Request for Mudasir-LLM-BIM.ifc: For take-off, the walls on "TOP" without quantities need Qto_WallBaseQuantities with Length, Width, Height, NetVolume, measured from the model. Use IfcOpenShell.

First a look at what the model holds.

```python
import ifcopenshell
import ifcopenshell.util.element
import ifcopenshell.util.unit

model = ifcopenshell.open("Mudasir-LLM-BIM.ifc")
print(model.schema)
for unit_type in ("LENGTHUNIT", "AREAUNIT", "VOLUMEUNIT"):
    print(unit_type, ifcopenshell.util.unit.calculate_unit_scale(model, unit_type))
storey = next(s for s in model.by_type("IfcBuildingStorey") if s.Name == "TOP")
walls = [e for e in ifcopenshell.util.element.get_decomposition(storey) if e.is_a("IfcWall")]
for e in sorted(walls, key=lambda e: e.id()):
    print(e.id(), e.is_a(), e.Name, list(ifcopenshell.util.element.get_psets(e, qtos_only=True)), sep=" | ")
```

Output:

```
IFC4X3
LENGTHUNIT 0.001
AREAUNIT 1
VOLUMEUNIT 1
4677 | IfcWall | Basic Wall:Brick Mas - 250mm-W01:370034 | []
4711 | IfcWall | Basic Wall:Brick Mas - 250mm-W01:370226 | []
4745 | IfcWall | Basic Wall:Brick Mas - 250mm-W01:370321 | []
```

```python
import ifcopenshell
import ifcopenshell.api.pset
import ifcopenshell.geom
import ifcopenshell.util.element
import ifcopenshell.util.shape
import ifcopenshell.util.unit

model = ifcopenshell.open("Mudasir-LLM-BIM.ifc")
unit_scale = ifcopenshell.util.unit.calculate_unit_scale(model)
volume_scale = ifcopenshell.util.unit.calculate_unit_scale(model, "VOLUMEUNIT")
settings = ifcopenshell.geom.settings()

storey = next(s for s in model.by_type("IfcBuildingStorey") if s.Name == "TOP")
walls = [e for e in ifcopenshell.util.element.get_decomposition(storey) if e.is_a("IfcWall")]

for e in sorted(walls, key=lambda e: e.id()):
    if ifcopenshell.util.element.get_psets(e, qtos_only=True, should_inherit=False):
        continue
    # Geometry comes back in metres, in the element's own axes.
    shape = ifcopenshell.geom.create_shape(settings, e)
    values = {
        "Length": ifcopenshell.util.shape.get_x(shape.geometry) / unit_scale,
        "Width": ifcopenshell.util.shape.get_y(shape.geometry) / unit_scale,
        "Height": ifcopenshell.util.shape.get_z(shape.geometry) / unit_scale,
        "NetVolume": ifcopenshell.util.shape.get_volume(shape.geometry) / volume_scale,
    }
    qto = ifcopenshell.api.pset.add_qto(model, product=e, name="Qto_WallBaseQuantities")
    ifcopenshell.api.pset.edit_qto(model, qto=qto, properties=values)
    print(e.id(), {k: round(v, 3) for k, v in values.items()})

model.write("Mudasir-LLM-BIM-out.ifc")
```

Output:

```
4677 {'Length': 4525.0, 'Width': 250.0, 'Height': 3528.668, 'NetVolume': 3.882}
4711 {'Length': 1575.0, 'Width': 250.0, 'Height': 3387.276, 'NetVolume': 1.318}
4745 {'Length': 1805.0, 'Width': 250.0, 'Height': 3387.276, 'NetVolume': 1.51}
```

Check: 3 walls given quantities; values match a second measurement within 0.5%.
